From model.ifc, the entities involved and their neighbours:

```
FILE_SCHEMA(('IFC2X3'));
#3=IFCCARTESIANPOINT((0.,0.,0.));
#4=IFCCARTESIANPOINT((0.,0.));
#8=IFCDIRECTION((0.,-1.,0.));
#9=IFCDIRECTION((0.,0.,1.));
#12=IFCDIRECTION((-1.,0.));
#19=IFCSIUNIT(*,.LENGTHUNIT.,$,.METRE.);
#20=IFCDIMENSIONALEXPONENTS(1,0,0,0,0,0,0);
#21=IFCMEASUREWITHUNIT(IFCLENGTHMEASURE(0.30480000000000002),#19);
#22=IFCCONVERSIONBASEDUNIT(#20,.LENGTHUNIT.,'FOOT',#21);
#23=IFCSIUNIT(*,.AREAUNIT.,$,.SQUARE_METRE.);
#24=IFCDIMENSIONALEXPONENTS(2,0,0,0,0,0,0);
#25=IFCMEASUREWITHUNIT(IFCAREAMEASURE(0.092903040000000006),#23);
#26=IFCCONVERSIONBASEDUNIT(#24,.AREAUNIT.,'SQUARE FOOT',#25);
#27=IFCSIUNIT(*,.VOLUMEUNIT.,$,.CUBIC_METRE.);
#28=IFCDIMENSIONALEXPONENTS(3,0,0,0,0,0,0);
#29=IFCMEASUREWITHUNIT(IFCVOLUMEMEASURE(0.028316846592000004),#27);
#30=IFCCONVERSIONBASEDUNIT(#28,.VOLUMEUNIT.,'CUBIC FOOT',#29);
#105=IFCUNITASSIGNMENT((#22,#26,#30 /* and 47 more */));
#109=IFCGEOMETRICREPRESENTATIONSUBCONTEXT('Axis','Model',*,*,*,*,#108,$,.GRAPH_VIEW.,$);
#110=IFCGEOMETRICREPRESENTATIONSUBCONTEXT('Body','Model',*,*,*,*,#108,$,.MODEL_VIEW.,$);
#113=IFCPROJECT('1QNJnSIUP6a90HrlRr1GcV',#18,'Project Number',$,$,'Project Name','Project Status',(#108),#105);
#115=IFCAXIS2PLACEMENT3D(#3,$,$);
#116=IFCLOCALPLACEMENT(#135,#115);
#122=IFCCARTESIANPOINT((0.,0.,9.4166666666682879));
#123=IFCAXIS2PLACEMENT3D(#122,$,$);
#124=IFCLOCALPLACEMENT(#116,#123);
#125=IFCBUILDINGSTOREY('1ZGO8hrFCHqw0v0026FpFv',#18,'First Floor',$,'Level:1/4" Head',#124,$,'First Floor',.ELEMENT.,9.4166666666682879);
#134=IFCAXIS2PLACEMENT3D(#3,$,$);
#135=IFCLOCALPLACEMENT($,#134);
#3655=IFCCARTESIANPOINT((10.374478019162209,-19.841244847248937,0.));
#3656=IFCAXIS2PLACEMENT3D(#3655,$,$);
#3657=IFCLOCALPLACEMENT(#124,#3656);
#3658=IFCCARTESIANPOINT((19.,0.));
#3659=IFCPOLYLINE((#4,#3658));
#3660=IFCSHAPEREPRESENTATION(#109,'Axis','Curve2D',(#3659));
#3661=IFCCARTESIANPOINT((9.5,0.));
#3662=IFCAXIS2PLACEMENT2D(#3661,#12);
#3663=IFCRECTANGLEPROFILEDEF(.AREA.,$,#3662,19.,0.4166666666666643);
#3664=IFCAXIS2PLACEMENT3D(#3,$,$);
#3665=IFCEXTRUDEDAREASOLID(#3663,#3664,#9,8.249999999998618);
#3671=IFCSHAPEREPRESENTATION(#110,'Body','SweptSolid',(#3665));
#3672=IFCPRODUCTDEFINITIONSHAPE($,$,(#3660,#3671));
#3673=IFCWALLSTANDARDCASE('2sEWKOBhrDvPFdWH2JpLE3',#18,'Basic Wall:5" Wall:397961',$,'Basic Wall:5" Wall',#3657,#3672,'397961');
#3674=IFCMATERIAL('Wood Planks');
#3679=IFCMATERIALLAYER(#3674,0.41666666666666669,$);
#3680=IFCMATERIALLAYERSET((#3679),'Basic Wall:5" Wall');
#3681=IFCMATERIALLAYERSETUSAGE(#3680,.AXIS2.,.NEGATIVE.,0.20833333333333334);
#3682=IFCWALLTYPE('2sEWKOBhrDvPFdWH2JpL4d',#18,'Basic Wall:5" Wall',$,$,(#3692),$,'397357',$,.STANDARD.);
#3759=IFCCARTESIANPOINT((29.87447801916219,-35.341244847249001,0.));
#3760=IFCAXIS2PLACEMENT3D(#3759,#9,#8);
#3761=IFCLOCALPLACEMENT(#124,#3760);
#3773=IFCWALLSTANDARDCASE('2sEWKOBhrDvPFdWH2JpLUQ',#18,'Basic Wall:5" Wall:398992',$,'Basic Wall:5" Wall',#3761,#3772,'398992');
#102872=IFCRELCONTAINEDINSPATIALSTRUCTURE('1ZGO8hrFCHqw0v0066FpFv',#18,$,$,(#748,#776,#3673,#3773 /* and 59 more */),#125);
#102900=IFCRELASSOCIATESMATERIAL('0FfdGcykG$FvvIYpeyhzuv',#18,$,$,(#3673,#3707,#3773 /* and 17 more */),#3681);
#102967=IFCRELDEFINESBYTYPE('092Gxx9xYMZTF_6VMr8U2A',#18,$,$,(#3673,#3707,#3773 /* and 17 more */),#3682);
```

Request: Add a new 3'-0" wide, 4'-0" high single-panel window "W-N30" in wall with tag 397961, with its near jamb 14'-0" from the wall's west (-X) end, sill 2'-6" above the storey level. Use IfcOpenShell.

```python
import numpy as np
import ifcopenshell
import ifcopenshell.api.feature
import ifcopenshell.api.geometry
import ifcopenshell.api.root
import ifcopenshell.api.spatial
import ifcopenshell.api.type
import ifcopenshell.geom
import ifcopenshell.util.element
import ifcopenshell.util.placement
import ifcopenshell.util.representation
import ifcopenshell.util.shape
import ifcopenshell.util.unit

model = ifcopenshell.open("model.ifc")
unit_scale = ifcopenshell.util.unit.calculate_unit_scale(model)
settings = ifcopenshell.geom.settings()


def volume(element):
    """Net volume in cubic metres, openings subtracted."""
    shape = ifcopenshell.geom.create_shape(settings, element)
    return ifcopenshell.util.shape.get_volume(shape.geometry)


wall = model.by_guid("2sEWKOBhrDvPFdWH2JpLE3")
storey = ifcopenshell.util.element.get_container(wall, ifc_class="IfcBuildingStorey")
context = ifcopenshell.util.representation.get_context(model, "Model", "Body", "MODEL_VIEW")
before = volume(wall)

width, height, from_end, sill = 0.9144, 1.2192, 4.2672, 0.762  # metres

# The wall runs along its own X axis, and the end named is its -X end.
wall_shape = ifcopenshell.geom.create_shape(settings, wall)
x, y, z = ifcopenshell.util.shape.get_vertices(wall_shape.geometry).T
start = x.min() + from_end
face, thickness = float(y.min()), float(y.max() - y.min())
wall_matrix = ifcopenshell.util.placement.get_local_placement(wall.ObjectPlacement)
level = ifcopenshell.util.placement.get_local_placement(storey.ObjectPlacement)[2, 3]


def in_wall(x, y):
    """Placement at x, y metres in the wall's axes, at sill height."""
    matrix = wall_matrix.copy()
    matrix[:, 3] = wall_matrix @ np.array([x / unit_scale, y / unit_scale, 0.0, 1.0])
    matrix[2, 3] = level + sill / unit_scale
    return matrix


# Opening: a box that overshoots both wall faces by 50 mm.
opening = ifcopenshell.api.root.create_entity(model, ifc_class="IfcOpeningElement")
box = ifcopenshell.api.geometry.add_wall_representation(
    model, context=context, length=width, height=height, thickness=thickness + 0.1
)
ifcopenshell.api.geometry.assign_representation(model, product=opening, representation=box)
ifcopenshell.api.geometry.edit_object_placement(model, product=opening, matrix=in_wall(start, face - 0.05), is_si=False)
ifcopenshell.api.feature.add_feature(model, feature=opening, element=wall)

window = ifcopenshell.api.root.create_entity(model, ifc_class="IfcWindow", name="W-N30")
window.OverallWidth, window.OverallHeight = width / unit_scale, height / unit_scale
body = ifcopenshell.api.geometry.add_window_representation(
    model,
    context=context,
    overall_width=window.OverallWidth,
    overall_height=window.OverallHeight,
    partition_type="SINGLE_PANEL",
)
ifcopenshell.api.geometry.assign_representation(model, product=window, representation=body)
ifcopenshell.api.spatial.assign_container(model, products=[window], relating_structure=storey)
fills = ifcopenshell.api.feature.add_filling(model, opening=opening, element=window)
fills.OwnerHistory = window.OwnerHistory  # required in IFC2X3

# IFC2X3 keeps the operation on the window style.
style = ifcopenshell.api.root.create_entity(model, ifc_class="IfcWindowStyle", name="W-N30")
style.OperationType, style.ConstructionType = "SINGLE_PANEL", "NOTDEFINED"
style.ParameterTakesPrecedence = style.Sizeable = False
ifcopenshell.api.type.assign_type(model, related_objects=[window], relating_type=style)

# Centre the window in the wall's thickness.
ifcopenshell.api.geometry.edit_object_placement(model, product=window, matrix=in_wall(start, face), is_si=False)
window_shape = ifcopenshell.geom.create_shape(settings, window)
depth = ifcopenshell.util.shape.get_vertices(window_shape.geometry)[:, 1]
offset = face + thickness / 2 - (depth.min() + depth.max()) / 2
ifcopenshell.api.geometry.edit_object_placement(model, product=window, matrix=in_wall(start, offset), is_si=False)

after = volume(wall)

print(f"wall volume {before:.3f} -> {after:.3f} m3")

model.write("model-out.ifc")
```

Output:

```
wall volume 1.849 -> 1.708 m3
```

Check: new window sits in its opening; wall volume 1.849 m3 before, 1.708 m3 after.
